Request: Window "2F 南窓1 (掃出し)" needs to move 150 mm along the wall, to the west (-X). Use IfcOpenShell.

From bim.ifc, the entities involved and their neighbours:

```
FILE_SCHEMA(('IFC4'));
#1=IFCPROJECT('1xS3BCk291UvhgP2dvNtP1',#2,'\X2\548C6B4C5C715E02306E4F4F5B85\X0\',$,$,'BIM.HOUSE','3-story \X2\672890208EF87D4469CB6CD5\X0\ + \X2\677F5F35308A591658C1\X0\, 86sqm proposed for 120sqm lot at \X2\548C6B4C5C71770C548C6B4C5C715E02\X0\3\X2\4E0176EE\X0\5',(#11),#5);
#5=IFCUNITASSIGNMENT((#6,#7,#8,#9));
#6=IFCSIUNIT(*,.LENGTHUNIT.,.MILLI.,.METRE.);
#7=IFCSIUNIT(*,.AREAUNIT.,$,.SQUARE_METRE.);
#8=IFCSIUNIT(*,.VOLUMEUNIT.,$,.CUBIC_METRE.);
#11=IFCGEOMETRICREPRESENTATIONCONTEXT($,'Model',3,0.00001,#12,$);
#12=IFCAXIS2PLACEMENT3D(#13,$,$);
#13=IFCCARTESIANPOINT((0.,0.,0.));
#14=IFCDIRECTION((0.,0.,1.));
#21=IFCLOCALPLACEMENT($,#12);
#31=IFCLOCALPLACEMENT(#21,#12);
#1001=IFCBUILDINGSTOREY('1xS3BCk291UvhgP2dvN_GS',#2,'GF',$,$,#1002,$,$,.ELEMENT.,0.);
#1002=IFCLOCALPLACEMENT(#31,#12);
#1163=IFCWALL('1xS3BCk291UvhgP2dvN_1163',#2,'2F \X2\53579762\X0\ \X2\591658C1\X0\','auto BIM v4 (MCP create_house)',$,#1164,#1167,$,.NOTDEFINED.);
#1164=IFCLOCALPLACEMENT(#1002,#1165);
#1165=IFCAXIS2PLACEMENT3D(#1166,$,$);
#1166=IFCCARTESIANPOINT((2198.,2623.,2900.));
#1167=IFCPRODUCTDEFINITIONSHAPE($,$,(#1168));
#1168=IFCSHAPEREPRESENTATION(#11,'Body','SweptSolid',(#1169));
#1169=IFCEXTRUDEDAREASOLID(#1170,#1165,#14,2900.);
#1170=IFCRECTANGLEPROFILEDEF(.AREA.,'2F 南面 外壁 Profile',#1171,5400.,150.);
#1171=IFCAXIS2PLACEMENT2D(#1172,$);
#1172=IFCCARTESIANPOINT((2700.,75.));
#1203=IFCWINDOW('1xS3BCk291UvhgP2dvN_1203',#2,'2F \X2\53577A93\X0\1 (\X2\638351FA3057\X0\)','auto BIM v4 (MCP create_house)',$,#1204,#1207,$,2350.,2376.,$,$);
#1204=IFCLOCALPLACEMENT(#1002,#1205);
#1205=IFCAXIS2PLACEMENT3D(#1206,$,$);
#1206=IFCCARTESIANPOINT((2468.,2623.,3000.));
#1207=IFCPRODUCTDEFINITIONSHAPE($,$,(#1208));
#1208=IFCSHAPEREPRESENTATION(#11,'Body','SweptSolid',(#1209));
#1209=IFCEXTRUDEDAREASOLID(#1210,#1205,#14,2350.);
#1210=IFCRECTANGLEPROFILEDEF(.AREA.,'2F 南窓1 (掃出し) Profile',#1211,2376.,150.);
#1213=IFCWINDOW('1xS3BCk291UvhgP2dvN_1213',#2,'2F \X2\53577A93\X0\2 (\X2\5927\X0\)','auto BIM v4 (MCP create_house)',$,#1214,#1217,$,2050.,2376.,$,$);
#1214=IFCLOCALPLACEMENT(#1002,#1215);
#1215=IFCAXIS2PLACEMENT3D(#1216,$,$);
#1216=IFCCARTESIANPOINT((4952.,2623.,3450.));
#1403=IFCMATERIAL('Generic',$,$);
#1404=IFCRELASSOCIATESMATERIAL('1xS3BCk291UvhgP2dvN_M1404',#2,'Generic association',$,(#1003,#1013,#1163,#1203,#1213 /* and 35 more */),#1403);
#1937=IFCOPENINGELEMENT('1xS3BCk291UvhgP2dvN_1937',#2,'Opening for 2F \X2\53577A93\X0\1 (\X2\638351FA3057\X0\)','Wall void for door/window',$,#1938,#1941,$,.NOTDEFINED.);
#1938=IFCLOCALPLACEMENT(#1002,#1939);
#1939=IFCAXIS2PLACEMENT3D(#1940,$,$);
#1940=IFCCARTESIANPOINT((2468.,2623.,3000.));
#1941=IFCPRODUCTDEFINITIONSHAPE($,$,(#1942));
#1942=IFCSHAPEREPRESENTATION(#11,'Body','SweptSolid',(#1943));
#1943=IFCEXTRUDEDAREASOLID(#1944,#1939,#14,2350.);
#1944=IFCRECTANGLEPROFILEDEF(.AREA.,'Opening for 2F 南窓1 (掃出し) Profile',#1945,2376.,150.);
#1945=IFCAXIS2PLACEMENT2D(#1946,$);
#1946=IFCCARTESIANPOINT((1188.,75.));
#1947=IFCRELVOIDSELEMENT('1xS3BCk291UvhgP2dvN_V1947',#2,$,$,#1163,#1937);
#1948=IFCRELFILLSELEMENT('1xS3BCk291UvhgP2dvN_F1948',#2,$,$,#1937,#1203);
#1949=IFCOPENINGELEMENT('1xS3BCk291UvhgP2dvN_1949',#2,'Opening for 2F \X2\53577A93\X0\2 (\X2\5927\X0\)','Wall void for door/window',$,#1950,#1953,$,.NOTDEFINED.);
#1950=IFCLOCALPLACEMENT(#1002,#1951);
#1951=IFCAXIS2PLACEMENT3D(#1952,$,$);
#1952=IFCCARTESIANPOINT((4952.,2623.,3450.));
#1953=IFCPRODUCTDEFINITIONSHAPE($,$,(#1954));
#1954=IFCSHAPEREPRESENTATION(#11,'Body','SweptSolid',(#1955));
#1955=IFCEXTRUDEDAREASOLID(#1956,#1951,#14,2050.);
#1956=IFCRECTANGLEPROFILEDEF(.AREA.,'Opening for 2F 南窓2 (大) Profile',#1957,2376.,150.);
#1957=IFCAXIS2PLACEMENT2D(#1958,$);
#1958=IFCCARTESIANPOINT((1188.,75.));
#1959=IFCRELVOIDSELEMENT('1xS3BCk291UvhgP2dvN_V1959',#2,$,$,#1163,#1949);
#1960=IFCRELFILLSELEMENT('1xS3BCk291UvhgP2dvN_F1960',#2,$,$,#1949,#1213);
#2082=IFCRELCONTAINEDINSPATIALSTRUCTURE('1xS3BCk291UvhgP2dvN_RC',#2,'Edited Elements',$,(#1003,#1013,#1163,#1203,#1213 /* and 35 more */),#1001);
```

```python
import ifcopenshell
import ifcopenshell.api.geometry
import ifcopenshell.util.placement

model = ifcopenshell.open("bim.ifc")

window = model.by_id(1203)
opening = window.FillsVoids[0].RelatingOpeningElement
wall = opening.VoidsElements[0].RelatingBuildingElement

wall_matrix = ifcopenshell.util.placement.get_local_placement(wall.ObjectPlacement)
shift = wall_matrix[:3, 0] * -150.0
before = ifcopenshell.util.placement.get_local_placement(window.ObjectPlacement)[:3, 3].copy()

# The window is not placed relative to its opening, so move both.
for product in (opening, window):
    matrix = ifcopenshell.util.placement.get_local_placement(product.ObjectPlacement)
    matrix[:3, 3] += shift
    ifcopenshell.api.geometry.edit_object_placement(model, product=product, matrix=matrix, is_si=False)

after = ifcopenshell.util.placement.get_local_placement(window.ObjectPlacement)[:3, 3]
print("window moved by", (after - before).round(3) + 0.0)

model.write("bim_updated.ifc")
```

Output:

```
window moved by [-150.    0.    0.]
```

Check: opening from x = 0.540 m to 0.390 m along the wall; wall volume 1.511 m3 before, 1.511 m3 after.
